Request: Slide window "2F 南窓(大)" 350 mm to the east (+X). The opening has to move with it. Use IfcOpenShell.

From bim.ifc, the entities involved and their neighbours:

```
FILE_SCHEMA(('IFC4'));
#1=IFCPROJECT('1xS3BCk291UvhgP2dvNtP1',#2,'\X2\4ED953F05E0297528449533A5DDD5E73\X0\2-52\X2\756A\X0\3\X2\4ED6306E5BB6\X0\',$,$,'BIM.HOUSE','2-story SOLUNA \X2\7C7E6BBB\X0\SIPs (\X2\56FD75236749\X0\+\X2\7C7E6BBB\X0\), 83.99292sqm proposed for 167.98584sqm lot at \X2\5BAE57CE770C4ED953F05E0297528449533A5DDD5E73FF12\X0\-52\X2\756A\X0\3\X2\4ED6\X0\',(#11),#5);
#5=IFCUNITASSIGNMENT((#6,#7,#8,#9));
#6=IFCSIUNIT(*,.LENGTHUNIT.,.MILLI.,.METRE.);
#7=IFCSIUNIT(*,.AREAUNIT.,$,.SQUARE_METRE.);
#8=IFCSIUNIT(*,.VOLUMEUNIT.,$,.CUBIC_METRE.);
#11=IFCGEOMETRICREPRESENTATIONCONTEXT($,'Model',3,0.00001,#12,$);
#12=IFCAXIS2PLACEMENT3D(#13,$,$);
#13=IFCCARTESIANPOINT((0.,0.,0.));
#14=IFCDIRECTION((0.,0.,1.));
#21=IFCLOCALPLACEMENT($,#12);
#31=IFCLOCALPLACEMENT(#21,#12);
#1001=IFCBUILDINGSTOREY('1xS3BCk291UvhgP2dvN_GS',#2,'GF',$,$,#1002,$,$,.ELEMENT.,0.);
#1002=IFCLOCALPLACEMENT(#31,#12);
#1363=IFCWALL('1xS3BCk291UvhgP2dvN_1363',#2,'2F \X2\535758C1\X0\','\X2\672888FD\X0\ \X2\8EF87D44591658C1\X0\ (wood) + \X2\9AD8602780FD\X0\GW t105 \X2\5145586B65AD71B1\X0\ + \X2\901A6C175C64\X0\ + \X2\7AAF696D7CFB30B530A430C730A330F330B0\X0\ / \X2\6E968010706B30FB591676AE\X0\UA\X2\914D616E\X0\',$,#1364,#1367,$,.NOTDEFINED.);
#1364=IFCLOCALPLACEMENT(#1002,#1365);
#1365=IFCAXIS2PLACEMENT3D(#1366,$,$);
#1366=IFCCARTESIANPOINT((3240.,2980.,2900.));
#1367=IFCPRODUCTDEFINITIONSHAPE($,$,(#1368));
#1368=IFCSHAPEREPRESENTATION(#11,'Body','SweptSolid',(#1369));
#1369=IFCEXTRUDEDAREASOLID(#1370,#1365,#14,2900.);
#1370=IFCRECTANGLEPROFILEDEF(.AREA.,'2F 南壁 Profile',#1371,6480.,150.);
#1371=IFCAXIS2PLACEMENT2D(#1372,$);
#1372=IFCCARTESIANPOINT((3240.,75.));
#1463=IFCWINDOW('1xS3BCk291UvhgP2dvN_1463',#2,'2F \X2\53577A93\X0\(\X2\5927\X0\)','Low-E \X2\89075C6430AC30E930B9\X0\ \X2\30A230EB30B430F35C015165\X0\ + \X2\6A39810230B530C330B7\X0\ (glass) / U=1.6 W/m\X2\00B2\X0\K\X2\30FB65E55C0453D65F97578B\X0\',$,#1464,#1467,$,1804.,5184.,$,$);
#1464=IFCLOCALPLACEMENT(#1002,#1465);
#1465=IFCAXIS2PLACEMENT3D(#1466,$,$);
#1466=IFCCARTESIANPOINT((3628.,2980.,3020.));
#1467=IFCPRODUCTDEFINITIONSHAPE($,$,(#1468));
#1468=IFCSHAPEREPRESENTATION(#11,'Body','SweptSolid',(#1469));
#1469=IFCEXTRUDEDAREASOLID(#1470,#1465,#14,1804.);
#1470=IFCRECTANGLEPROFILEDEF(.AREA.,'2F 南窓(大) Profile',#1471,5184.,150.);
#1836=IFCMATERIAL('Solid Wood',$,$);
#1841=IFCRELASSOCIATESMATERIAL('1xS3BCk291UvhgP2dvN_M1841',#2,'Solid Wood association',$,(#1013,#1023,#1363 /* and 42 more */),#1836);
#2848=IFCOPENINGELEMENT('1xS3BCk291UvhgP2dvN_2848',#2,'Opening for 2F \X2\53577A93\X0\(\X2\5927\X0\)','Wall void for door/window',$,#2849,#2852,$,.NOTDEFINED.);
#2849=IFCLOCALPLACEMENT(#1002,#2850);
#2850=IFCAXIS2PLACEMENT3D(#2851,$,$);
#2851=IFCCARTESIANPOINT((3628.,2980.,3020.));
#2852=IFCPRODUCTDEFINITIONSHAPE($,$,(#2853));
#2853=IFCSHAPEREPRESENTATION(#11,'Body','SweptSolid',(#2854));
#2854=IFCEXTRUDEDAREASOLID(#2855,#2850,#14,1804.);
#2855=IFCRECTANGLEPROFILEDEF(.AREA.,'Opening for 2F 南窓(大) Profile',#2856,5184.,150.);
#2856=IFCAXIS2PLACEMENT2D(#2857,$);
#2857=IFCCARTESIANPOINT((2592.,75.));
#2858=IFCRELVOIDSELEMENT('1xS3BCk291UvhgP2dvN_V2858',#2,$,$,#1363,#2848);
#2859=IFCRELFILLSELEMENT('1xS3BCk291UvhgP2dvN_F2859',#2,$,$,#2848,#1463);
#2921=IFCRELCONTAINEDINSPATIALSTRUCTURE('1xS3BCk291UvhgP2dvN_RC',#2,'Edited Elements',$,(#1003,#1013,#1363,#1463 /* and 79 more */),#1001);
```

```python
import ifcopenshell
import ifcopenshell.api.geometry
import ifcopenshell.util.placement
import ifcopenshell.util.unit

model = ifcopenshell.open("bim.ifc")
unit_scale = ifcopenshell.util.unit.calculate_unit_scale(model)

window = model.by_id(1463)
opening = window.FillsVoids[0].RelatingOpeningElement
wall = opening.VoidsElements[0].RelatingBuildingElement

wall_matrix = ifcopenshell.util.placement.get_local_placement(wall.ObjectPlacement)
shift = wall_matrix[:3, 0] * 0.35 / unit_scale
before = ifcopenshell.util.placement.get_local_placement(window.ObjectPlacement)[:3, 3].copy()

# The window is not placed relative to its opening, so move both.
for product in (opening, window):
    matrix = ifcopenshell.util.placement.get_local_placement(product.ObjectPlacement)
    matrix[:3, 3] += shift
    ifcopenshell.api.geometry.edit_object_placement(model, product=product, matrix=matrix, is_si=False)

after = ifcopenshell.util.placement.get_local_placement(window.ObjectPlacement)[:3, 3]
print("window moved by", (after - before).round(3) + 0.0)

model.write("bim_updated.ifc")
```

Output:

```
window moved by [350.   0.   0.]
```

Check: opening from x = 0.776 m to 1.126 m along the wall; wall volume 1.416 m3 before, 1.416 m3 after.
